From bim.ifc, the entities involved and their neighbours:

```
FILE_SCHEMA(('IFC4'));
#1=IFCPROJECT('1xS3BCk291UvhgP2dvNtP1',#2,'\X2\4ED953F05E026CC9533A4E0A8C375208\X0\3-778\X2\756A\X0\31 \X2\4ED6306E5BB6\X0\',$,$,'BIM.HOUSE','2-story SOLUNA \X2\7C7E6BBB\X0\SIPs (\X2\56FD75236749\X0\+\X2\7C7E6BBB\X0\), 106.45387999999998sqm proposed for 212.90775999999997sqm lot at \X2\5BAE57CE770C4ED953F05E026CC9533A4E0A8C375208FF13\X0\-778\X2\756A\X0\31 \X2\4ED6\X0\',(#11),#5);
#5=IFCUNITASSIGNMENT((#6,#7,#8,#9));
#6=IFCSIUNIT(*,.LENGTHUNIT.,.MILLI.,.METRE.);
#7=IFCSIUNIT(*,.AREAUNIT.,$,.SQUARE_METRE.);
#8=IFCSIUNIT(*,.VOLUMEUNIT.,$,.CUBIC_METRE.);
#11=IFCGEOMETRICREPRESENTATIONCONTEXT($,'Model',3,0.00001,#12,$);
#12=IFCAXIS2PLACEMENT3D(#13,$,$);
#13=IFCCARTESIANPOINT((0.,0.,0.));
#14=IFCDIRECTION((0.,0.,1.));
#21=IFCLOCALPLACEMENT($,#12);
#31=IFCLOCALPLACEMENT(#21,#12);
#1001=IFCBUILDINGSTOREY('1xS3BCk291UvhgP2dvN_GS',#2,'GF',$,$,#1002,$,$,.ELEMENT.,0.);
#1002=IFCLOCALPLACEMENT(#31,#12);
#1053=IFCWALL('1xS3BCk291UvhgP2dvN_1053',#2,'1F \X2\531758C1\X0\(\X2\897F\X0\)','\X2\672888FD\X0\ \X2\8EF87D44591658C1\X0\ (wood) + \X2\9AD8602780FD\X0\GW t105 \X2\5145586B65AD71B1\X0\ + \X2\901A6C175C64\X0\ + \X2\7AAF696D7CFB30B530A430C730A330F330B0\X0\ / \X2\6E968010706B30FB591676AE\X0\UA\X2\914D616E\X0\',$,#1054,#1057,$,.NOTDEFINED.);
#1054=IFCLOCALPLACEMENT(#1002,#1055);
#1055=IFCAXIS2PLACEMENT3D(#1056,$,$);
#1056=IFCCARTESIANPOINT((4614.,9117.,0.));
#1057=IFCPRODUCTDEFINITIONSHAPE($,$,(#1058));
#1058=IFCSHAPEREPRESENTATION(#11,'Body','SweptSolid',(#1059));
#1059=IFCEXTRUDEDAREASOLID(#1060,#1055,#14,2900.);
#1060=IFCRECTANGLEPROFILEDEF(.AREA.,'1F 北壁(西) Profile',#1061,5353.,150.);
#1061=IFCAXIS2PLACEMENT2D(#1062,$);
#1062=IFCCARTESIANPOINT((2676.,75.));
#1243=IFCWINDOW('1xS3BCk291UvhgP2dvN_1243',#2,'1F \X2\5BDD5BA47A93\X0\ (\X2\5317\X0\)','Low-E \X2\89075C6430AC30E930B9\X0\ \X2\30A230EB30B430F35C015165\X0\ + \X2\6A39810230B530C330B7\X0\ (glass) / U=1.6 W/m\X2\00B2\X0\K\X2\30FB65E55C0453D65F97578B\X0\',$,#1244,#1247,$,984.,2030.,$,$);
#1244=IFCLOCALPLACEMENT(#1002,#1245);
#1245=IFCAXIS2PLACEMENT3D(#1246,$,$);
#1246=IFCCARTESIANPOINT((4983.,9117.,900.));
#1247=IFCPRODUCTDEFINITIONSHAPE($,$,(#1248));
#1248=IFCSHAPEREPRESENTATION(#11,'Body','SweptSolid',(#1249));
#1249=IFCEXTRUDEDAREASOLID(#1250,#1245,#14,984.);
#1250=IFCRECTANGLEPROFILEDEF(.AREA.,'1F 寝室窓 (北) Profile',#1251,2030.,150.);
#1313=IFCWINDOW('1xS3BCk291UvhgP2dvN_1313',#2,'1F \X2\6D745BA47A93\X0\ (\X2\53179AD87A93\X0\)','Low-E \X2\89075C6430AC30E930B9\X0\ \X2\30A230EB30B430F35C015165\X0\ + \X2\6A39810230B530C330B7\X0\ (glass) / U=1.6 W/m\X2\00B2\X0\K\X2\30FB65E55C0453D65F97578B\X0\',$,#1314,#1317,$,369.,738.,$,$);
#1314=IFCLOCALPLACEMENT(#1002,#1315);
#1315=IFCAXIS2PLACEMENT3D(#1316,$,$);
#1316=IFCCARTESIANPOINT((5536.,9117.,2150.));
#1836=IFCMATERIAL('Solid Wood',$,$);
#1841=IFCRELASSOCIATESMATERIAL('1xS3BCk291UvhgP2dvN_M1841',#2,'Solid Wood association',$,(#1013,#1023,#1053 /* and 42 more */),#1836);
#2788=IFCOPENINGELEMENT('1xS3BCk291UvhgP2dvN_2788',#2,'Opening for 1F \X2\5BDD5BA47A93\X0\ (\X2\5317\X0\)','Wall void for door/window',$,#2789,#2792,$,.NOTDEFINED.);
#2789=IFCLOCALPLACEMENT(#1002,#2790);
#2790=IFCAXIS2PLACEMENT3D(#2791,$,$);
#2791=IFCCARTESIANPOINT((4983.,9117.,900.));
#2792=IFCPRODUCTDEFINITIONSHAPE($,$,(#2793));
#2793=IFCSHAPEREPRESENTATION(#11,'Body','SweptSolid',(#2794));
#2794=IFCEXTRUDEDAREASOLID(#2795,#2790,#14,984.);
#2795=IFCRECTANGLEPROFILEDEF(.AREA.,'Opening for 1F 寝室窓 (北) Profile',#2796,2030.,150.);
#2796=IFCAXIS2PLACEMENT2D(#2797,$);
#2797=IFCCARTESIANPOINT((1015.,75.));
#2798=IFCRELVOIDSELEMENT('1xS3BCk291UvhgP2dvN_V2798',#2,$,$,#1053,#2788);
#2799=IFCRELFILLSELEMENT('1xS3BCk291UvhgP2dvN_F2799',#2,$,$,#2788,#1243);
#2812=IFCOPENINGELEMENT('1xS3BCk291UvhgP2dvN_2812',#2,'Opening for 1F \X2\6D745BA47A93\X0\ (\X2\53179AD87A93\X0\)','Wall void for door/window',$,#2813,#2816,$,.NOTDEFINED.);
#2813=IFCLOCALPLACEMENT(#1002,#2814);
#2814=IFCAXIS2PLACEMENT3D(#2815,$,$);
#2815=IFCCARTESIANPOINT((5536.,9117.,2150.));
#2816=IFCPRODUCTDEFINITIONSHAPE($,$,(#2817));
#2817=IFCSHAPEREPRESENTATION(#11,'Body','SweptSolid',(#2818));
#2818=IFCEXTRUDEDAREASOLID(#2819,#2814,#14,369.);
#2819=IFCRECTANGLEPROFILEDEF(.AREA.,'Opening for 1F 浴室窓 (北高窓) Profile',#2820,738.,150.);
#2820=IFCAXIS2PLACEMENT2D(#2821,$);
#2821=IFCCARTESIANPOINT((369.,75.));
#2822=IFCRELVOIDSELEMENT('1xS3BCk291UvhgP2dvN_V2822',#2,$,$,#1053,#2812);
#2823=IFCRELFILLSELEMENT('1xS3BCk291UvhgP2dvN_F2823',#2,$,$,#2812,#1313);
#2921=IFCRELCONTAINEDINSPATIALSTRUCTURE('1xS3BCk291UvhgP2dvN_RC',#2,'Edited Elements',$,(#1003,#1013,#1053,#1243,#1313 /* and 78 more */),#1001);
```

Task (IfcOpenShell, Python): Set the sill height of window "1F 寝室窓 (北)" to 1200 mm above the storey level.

```python
import numpy as np
import ifcopenshell
import ifcopenshell.api.geometry
import ifcopenshell.geom
import ifcopenshell.util.element
import ifcopenshell.util.placement
import ifcopenshell.util.shape
import ifcopenshell.util.unit

model = ifcopenshell.open("bim.ifc")
unit_scale = ifcopenshell.util.unit.calculate_unit_scale(model)

window = model.by_guid("1xS3BCk291UvhgP2dvN_1243")
opening = window.FillsVoids[0].RelatingOpeningElement
storey = ifcopenshell.util.element.get_container(window, ifc_class="IfcBuildingStorey")
level = ifcopenshell.util.placement.get_local_placement(storey.ObjectPlacement)[2, 3]

# The opening's origin need not be at the sill, so measure its lowest point.
shape = ifcopenshell.geom.create_shape(ifcopenshell.geom.settings(), opening)
bottom = ifcopenshell.util.shape.get_shape_bottom_elevation(shape, shape.geometry) / unit_scale
dz = level + 1200.0 - bottom

shift = np.array([0.0, 0.0, dz])
# The window is not placed relative to its opening, so move both.
for product in (opening, window):
    matrix = ifcopenshell.util.placement.get_local_placement(product.ObjectPlacement)
    matrix[:3, 3] += shift
    ifcopenshell.api.geometry.edit_object_placement(model, product=product, matrix=matrix, is_si=False)

print(f"moved by {dz * unit_scale:+.3f} m")

model.write("bim-out.ifc")
```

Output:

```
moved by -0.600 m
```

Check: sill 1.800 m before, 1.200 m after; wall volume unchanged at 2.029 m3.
